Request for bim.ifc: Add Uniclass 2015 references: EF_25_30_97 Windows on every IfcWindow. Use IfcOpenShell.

First a look at what the model holds.

```python
import ifcopenshell

model = ifcopenshell.open("bim.ifc")
print(model.schema)
print("classifications:", [c.Name for c in model.by_type("IfcClassification")])
for ifc_class in ("IfcDoor", "IfcRoof", "IfcStair", "IfcWall", "IfcWindow"):
    print(ifc_class, len(model.by_type(ifc_class)))
```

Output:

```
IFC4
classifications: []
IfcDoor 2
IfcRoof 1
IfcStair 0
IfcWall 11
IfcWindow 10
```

```python
import ifcopenshell
import ifcopenshell.api.classification

model = ifcopenshell.open("bim.ifc")

system = ifcopenshell.api.classification.add_classification(model, classification="Uniclass 2015")

codes = {
    "IfcWindow": ("EF_25_30_97", "Windows"),
}
for ifc_class, (code, name) in codes.items():
    products = model.by_type(ifc_class)
    ifcopenshell.api.classification.add_reference(
        model, products=products, classification=system, identification=code, name=name
    )
    print(code, len(products))

model.write("bim_v2.ifc")
```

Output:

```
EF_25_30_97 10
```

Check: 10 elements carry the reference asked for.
